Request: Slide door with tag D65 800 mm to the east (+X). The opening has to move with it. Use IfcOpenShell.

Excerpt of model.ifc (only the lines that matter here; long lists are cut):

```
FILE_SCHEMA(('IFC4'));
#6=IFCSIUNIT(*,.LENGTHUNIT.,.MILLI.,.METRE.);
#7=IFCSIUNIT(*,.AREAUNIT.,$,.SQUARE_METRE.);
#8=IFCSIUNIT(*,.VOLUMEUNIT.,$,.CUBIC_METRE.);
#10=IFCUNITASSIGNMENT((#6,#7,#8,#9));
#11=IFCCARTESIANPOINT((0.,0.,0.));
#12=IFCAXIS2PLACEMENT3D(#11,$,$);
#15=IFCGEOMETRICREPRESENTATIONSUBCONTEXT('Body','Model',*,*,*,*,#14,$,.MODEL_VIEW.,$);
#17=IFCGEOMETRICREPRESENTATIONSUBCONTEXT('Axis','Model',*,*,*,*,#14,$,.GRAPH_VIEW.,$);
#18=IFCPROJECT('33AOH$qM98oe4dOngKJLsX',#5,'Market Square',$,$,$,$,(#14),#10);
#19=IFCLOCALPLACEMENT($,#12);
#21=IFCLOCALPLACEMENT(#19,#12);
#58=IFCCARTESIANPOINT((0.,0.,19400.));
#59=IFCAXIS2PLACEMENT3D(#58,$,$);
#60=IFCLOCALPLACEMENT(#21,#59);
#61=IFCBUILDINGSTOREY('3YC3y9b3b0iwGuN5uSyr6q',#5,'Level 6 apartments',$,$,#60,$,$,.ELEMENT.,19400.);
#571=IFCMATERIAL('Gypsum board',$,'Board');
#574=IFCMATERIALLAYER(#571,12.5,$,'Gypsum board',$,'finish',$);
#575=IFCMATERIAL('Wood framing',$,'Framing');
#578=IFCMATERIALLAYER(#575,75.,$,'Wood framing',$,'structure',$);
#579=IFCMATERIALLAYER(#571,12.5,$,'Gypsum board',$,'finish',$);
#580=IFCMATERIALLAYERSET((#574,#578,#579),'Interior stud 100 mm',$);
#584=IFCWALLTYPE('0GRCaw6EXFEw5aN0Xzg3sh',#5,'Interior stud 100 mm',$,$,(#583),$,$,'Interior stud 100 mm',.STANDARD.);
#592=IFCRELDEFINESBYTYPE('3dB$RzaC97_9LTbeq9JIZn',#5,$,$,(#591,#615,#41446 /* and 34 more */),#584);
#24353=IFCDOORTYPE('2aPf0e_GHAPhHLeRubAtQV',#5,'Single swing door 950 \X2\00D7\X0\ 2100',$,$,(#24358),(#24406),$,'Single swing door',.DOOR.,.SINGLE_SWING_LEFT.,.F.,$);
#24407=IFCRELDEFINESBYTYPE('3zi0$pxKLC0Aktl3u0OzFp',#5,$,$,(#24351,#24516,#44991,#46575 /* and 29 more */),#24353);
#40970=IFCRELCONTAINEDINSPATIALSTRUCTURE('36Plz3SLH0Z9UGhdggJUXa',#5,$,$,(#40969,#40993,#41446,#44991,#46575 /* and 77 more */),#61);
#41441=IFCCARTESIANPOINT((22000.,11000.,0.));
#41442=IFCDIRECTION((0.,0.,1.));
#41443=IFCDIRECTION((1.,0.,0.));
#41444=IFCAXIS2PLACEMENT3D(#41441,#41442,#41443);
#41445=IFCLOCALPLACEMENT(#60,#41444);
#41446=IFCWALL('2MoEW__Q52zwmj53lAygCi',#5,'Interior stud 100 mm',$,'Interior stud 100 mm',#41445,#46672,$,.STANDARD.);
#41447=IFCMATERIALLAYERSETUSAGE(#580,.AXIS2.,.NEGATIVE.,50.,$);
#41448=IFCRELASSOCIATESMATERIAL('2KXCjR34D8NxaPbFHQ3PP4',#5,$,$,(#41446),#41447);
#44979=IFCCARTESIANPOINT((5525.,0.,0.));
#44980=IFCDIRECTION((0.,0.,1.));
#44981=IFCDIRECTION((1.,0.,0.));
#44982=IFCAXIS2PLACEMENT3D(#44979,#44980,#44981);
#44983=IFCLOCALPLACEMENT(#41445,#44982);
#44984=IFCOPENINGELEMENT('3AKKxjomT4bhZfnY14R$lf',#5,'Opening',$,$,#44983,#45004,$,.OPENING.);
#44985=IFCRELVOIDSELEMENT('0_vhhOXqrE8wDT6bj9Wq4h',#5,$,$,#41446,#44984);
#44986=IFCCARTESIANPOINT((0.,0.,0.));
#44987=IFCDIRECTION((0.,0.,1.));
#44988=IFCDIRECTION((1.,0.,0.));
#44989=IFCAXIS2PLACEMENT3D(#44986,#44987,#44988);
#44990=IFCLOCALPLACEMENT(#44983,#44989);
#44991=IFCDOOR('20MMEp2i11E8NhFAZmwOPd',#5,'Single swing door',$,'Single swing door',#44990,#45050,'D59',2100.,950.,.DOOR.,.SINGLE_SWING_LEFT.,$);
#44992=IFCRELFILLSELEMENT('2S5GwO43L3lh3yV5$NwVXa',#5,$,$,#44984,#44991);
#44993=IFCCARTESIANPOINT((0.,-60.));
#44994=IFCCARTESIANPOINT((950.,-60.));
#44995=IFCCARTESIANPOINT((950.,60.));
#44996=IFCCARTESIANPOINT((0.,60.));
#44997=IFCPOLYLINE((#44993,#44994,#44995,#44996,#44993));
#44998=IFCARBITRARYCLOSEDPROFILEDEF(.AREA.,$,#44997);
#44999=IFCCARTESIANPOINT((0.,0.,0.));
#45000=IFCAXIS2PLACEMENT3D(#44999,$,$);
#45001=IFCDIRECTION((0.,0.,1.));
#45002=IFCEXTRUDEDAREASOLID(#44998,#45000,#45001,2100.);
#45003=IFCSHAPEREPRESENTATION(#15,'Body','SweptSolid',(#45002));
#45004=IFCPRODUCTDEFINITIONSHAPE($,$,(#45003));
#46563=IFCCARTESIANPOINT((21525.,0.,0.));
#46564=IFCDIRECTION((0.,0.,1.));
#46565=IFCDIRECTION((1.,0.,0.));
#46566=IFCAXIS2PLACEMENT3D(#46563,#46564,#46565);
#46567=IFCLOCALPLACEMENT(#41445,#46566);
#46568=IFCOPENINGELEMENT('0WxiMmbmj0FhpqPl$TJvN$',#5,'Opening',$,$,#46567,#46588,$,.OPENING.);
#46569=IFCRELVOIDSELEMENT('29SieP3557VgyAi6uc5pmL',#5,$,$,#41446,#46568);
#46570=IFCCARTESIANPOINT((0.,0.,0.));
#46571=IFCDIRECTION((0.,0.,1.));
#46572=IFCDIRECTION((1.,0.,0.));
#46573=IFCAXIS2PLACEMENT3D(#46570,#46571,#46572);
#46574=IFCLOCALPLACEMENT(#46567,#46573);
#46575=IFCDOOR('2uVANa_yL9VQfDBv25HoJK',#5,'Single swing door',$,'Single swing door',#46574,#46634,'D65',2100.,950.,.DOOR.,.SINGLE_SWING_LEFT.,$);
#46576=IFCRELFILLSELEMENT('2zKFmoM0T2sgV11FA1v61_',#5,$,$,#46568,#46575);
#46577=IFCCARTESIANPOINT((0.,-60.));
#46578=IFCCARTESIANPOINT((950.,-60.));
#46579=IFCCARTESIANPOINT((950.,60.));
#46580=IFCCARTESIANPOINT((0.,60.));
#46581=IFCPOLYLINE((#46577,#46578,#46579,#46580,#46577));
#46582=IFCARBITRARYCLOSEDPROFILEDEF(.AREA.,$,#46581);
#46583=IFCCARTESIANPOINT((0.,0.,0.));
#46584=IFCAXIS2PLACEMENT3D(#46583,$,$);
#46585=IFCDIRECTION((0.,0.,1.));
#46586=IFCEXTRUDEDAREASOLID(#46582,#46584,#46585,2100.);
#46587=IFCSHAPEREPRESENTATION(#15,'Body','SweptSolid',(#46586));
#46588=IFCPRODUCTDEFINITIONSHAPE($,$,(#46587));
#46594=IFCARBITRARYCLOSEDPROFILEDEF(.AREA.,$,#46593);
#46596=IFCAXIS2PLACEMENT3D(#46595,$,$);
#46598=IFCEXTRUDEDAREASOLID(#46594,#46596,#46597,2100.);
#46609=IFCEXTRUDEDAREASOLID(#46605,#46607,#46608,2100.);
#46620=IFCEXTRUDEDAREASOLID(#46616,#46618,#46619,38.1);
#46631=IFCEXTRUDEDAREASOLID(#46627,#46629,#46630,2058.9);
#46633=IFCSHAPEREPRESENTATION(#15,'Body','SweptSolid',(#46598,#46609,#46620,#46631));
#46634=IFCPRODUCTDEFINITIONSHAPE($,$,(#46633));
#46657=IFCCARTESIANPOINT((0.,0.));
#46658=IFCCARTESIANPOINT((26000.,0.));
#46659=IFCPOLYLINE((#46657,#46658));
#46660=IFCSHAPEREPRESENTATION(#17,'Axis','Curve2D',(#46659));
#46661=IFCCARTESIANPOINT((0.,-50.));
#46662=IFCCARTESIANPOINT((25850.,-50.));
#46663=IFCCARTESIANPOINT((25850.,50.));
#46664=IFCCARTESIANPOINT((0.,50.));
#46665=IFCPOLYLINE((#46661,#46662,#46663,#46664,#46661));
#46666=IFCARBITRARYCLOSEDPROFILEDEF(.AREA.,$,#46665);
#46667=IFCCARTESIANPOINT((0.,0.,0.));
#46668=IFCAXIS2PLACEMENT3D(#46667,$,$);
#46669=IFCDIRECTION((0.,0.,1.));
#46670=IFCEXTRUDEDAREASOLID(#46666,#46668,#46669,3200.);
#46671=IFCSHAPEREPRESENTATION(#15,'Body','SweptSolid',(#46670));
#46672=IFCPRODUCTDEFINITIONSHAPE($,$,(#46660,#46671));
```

```python
import ifcopenshell
import ifcopenshell.api.geometry
import ifcopenshell.util.placement
import ifcopenshell.util.unit

model = ifcopenshell.open("model.ifc")
unit_scale = ifcopenshell.util.unit.calculate_unit_scale(model)

door = model.by_id(46575)
opening = door.FillsVoids[0].RelatingOpeningElement
wall = opening.VoidsElements[0].RelatingBuildingElement

wall_matrix = ifcopenshell.util.placement.get_local_placement(wall.ObjectPlacement)
shift = wall_matrix[:3, 0] * 0.8 / unit_scale
before = ifcopenshell.util.placement.get_local_placement(door.ObjectPlacement)[:3, 3].copy()

# The door is placed relative to its opening, so it follows when the opening moves.
matrix = ifcopenshell.util.placement.get_local_placement(opening.ObjectPlacement)
matrix[:3, 3] += shift
ifcopenshell.api.geometry.edit_object_placement(
    model, product=opening, matrix=matrix, is_si=False, should_transform_children=True
)

after = ifcopenshell.util.placement.get_local_placement(door.ObjectPlacement)[:3, 3]
print("door moved by", (after - before).round(3) + 0.0)

model.write("model_v2.ifc")
```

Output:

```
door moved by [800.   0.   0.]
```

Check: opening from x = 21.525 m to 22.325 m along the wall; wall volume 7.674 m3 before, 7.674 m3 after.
